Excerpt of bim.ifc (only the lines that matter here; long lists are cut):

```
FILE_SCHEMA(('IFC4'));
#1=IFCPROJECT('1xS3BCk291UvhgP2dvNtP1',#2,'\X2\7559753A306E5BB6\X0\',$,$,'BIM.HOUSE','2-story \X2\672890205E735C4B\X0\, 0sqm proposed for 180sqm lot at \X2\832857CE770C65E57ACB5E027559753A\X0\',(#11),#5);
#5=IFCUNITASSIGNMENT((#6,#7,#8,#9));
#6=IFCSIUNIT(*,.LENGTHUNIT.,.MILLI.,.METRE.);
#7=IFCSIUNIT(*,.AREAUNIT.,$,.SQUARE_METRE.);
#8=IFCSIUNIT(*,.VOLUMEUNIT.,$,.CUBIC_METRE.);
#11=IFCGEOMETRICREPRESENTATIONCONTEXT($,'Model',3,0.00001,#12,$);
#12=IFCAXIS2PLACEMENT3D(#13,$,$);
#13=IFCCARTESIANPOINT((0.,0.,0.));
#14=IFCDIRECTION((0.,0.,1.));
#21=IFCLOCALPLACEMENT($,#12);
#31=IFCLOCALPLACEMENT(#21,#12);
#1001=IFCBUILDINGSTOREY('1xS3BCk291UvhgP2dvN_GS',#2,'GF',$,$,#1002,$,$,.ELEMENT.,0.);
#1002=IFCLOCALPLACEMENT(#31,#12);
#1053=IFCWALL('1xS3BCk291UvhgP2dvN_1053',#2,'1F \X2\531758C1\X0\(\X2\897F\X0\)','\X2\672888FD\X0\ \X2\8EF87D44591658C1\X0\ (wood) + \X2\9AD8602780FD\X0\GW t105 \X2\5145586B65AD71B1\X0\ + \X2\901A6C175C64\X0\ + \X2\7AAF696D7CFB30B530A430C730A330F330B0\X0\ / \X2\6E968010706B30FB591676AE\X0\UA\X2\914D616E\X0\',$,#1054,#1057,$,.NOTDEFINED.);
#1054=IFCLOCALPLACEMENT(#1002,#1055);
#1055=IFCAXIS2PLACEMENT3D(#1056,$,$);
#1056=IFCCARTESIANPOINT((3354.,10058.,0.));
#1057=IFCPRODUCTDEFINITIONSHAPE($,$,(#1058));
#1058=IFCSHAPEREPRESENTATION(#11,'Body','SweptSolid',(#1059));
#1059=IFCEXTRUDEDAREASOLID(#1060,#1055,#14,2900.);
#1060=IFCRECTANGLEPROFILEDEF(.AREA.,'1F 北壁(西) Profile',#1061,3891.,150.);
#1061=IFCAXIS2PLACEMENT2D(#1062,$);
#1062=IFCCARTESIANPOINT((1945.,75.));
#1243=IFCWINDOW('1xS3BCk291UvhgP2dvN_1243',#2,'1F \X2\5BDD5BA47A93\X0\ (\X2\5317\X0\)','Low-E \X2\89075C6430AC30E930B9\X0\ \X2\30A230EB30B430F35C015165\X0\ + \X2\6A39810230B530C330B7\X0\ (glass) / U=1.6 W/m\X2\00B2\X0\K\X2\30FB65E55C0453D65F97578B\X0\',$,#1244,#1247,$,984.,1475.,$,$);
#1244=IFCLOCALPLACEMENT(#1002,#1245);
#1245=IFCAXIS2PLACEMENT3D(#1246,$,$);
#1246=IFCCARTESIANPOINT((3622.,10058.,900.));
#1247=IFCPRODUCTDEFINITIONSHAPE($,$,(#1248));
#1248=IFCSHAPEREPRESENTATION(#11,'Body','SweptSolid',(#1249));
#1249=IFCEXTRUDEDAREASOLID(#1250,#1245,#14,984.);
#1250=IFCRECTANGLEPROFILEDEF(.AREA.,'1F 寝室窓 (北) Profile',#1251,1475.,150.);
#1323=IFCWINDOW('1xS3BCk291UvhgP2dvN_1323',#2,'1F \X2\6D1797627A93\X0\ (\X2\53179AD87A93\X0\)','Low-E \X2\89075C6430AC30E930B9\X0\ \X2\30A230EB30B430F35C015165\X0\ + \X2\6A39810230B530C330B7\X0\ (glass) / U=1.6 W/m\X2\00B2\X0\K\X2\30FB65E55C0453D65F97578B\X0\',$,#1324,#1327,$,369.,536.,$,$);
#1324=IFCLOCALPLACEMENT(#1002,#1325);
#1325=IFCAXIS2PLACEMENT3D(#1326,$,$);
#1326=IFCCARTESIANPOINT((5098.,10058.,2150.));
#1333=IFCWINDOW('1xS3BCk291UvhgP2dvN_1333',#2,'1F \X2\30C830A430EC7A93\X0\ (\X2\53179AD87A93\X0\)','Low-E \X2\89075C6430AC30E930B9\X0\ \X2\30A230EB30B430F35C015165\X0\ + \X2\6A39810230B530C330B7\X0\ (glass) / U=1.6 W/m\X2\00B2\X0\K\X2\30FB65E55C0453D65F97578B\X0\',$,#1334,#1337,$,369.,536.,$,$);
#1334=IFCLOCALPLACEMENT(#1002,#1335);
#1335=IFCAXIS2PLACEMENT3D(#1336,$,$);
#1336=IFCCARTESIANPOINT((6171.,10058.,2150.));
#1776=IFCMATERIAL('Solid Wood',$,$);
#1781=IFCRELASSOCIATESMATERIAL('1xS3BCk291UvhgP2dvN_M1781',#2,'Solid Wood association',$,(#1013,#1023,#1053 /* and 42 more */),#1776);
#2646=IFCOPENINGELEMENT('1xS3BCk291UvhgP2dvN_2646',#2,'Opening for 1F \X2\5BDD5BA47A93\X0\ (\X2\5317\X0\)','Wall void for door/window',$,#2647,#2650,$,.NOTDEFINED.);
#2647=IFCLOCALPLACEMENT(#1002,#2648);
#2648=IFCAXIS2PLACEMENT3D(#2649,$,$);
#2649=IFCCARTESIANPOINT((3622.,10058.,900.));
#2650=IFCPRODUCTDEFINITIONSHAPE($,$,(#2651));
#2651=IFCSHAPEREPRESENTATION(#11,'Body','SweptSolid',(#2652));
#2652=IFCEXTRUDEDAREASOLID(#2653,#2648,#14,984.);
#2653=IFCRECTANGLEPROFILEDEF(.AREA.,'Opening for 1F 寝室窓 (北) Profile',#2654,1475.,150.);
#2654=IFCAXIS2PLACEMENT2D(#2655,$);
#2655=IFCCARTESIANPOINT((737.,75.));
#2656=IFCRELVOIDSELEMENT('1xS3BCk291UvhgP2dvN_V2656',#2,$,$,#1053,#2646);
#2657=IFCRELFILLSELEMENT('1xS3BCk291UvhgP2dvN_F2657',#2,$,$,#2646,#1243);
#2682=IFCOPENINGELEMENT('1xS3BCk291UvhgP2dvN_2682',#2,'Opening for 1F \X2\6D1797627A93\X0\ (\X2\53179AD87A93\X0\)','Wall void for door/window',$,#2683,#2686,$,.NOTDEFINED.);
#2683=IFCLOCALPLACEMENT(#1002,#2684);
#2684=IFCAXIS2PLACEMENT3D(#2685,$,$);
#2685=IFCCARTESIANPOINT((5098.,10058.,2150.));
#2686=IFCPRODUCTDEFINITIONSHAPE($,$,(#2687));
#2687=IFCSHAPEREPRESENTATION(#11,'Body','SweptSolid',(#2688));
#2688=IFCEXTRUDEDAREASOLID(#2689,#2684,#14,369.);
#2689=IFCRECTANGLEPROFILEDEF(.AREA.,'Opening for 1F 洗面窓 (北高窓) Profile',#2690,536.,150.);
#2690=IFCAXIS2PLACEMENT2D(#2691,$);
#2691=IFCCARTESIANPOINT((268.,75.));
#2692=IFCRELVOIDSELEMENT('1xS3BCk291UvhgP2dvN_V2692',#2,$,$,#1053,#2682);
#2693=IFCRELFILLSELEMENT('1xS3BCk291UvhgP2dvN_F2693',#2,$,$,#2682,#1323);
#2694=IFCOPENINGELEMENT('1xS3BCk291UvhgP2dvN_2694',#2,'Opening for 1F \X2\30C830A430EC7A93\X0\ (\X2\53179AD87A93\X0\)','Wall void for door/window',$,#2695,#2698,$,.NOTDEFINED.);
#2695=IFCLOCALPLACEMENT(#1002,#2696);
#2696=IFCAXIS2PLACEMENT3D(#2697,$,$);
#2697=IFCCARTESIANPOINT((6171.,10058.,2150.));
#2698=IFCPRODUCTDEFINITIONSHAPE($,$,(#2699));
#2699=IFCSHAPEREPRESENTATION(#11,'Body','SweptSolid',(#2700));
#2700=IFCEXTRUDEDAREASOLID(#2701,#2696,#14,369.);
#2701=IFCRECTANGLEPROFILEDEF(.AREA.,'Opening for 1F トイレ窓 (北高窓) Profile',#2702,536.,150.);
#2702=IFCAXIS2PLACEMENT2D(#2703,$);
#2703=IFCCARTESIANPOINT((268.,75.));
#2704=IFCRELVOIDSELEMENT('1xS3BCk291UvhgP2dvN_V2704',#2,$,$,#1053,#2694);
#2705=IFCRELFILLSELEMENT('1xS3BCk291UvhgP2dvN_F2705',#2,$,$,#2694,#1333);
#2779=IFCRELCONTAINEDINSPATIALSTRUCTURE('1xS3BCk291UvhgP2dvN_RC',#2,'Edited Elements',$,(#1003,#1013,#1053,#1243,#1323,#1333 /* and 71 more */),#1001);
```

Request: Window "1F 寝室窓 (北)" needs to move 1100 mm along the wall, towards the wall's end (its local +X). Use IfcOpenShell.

```python
import ifcopenshell
import ifcopenshell.api.geometry
import ifcopenshell.util.placement
import ifcopenshell.util.unit

model = ifcopenshell.open("bim.ifc")
unit_scale = ifcopenshell.util.unit.calculate_unit_scale(model)

window = model.by_id(1243)
opening = window.FillsVoids[0].RelatingOpeningElement
wall = opening.VoidsElements[0].RelatingBuildingElement

wall_matrix = ifcopenshell.util.placement.get_local_placement(wall.ObjectPlacement)
shift = wall_matrix[:3, 0] * 1.1 / unit_scale
before = ifcopenshell.util.placement.get_local_placement(window.ObjectPlacement)[:3, 3].copy()

# The window is not placed relative to its opening, so move both.
for product in (opening, window):
    matrix = ifcopenshell.util.placement.get_local_placement(product.ObjectPlacement)
    matrix[:3, 3] += shift
    ifcopenshell.api.geometry.edit_object_placement(model, product=product, matrix=matrix, is_si=False)

after = ifcopenshell.util.placement.get_local_placement(window.ObjectPlacement)[:3, 3]
print("window moved by", (after - before).round(3) + 0.0)

model.write("bim_edited.ifc")
```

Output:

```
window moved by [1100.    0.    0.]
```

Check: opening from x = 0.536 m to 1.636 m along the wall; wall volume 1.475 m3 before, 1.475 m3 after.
